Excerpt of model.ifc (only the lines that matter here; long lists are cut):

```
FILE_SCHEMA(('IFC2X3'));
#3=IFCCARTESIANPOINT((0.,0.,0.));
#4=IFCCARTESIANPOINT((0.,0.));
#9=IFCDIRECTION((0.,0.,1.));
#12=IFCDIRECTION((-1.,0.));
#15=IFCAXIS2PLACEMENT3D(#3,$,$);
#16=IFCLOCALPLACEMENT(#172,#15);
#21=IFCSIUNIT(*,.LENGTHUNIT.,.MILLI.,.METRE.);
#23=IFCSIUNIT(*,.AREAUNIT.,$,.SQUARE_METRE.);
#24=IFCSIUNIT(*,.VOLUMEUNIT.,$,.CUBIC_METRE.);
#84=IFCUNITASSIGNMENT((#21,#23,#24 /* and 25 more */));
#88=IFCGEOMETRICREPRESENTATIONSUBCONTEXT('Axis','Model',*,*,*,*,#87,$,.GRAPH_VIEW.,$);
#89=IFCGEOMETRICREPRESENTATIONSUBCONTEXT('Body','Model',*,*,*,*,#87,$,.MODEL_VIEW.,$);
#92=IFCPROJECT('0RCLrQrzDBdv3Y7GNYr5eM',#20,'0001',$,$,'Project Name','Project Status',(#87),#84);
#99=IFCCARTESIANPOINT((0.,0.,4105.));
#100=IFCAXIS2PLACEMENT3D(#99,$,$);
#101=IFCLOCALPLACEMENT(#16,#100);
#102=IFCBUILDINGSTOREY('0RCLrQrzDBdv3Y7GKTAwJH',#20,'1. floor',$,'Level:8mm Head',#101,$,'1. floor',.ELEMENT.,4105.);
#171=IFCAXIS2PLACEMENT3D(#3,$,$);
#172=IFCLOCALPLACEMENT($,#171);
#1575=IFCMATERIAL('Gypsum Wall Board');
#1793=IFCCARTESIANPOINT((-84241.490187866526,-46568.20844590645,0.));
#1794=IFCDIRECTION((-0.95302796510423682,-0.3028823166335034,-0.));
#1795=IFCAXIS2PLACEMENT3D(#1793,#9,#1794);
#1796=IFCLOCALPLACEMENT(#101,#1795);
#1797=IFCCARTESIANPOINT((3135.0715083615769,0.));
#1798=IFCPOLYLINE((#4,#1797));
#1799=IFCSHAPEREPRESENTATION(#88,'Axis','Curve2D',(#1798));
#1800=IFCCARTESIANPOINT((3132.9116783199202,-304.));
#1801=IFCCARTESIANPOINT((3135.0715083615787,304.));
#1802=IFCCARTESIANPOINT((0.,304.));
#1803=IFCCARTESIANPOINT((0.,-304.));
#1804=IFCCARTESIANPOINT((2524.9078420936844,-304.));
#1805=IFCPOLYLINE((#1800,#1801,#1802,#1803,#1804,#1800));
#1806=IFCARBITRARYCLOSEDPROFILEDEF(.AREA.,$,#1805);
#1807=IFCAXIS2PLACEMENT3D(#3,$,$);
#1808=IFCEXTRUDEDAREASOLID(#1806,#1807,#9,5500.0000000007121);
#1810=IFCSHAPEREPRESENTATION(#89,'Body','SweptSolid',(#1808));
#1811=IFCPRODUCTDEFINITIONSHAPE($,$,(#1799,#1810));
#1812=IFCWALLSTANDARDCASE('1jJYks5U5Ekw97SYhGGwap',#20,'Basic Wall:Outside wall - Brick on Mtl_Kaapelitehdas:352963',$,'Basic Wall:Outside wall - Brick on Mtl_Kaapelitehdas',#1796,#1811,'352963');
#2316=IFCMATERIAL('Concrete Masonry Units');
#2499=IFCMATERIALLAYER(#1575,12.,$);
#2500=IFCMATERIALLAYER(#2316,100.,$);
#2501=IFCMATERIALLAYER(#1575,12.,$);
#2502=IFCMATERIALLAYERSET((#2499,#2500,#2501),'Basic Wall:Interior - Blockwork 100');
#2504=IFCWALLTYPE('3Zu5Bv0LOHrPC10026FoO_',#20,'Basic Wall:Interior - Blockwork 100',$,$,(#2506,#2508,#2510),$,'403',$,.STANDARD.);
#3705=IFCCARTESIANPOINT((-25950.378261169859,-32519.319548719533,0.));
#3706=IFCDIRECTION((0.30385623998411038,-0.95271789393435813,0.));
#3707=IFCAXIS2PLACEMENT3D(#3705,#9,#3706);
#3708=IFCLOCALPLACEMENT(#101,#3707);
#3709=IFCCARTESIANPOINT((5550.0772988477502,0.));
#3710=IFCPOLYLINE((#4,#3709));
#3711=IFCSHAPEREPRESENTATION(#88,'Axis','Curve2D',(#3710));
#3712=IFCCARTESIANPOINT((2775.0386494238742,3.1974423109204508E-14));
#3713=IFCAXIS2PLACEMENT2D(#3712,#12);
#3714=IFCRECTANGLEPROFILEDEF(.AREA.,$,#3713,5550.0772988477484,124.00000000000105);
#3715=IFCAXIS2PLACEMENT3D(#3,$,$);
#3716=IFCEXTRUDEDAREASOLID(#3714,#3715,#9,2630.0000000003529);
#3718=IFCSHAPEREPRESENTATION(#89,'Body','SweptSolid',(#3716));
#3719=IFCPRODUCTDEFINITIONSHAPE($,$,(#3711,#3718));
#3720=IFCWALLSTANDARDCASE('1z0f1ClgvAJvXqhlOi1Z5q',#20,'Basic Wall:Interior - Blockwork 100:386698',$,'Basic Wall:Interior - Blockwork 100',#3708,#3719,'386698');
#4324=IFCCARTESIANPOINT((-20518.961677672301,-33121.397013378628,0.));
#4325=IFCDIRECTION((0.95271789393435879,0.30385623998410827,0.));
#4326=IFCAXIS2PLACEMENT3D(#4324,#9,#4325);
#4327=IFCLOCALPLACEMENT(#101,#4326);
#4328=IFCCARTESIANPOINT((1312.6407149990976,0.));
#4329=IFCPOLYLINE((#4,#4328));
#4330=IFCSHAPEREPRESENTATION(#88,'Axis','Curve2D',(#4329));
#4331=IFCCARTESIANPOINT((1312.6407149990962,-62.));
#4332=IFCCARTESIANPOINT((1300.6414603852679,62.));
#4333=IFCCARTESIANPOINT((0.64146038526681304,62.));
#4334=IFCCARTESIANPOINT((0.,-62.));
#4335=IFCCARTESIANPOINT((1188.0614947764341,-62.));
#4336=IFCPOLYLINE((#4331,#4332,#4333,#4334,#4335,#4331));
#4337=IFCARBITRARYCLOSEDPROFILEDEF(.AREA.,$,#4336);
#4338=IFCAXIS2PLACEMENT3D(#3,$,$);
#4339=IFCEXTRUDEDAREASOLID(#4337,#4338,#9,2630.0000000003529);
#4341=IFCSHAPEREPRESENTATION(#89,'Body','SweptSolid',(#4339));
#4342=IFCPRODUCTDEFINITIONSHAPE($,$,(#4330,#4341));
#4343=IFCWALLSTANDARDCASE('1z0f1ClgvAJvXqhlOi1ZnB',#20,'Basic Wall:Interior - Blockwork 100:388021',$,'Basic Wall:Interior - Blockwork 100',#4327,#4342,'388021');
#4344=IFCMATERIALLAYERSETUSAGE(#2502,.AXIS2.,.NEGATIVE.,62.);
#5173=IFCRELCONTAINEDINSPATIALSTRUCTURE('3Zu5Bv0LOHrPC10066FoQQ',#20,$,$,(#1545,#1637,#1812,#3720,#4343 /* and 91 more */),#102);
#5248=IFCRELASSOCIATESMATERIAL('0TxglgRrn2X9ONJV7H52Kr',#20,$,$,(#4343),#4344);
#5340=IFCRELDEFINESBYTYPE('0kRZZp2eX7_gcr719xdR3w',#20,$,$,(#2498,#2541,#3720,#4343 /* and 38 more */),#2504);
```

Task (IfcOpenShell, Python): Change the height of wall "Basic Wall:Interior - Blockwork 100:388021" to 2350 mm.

```python
import ifcopenshell
import ifcopenshell.geom
import ifcopenshell.util.representation
import ifcopenshell.util.shape

model = ifcopenshell.open("model.ifc")
settings = ifcopenshell.geom.settings()


def volume(element):
    """Net volume in cubic metres, openings subtracted."""
    shape = ifcopenshell.geom.create_shape(settings, element)
    return ifcopenshell.util.shape.get_volume(shape.geometry)


wall = model.by_guid("1z0f1ClgvAJvXqhlOi1ZnB")
before = volume(wall)

body = ifcopenshell.util.representation.get_representation(wall, "Model", "Body")
solid = body.Items[0]
old_height = solid.Depth
solid.Depth = 2350.0
after = volume(wall)

print(f"height {old_height:g} -> {solid.Depth:g}, volume {before:.3f} -> {after:.3f} m3")

model.write("model_edited.ifc")
```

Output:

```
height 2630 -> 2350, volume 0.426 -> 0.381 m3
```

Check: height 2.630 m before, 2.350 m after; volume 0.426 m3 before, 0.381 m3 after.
